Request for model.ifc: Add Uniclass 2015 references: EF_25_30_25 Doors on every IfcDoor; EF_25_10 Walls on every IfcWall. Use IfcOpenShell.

First a look at what the model holds.

```python
import ifcopenshell

model = ifcopenshell.open("model.ifc")
print(model.schema)
print("classifications:", [c.Name for c in model.by_type("IfcClassification")])
for ifc_class in ("IfcDoor", "IfcRoof", "IfcStair", "IfcWall", "IfcWindow"):
    print(ifc_class, len(model.by_type(ifc_class)))
```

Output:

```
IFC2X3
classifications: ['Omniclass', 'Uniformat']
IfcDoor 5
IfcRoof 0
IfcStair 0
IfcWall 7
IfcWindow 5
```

```python
import ifcopenshell
import ifcopenshell.api.classification

model = ifcopenshell.open("model.ifc")

# IFC2X3 requires Source and Edition and has no link from the project to the system.
system = model.create_entity("IfcClassification", Source="NBS", Edition="2015", Name="Uniclass 2015")

codes = {
    "IfcDoor": ("EF_25_30_25", "Doors"),
    "IfcWall": ("EF_25_10", "Walls"),
}
for ifc_class, (code, name) in codes.items():
    products = model.by_type(ifc_class)
    ifcopenshell.api.classification.add_reference(
        model, products=products, classification=system, identification=code, name=name
    )
    print(code, len(products))

model.write("model_rev.ifc")
```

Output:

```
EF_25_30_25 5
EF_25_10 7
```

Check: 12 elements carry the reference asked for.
